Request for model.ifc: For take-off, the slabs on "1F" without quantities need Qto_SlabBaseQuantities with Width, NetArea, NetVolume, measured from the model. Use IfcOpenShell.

First a look at what the model holds.

```python
import ifcopenshell
import ifcopenshell.util.element
import ifcopenshell.util.unit

model = ifcopenshell.open("model.ifc")
print(model.schema)
for unit_type in ("LENGTHUNIT", "AREAUNIT", "VOLUMEUNIT"):
    print(unit_type, ifcopenshell.util.unit.calculate_unit_scale(model, unit_type))
storey = next(s for s in model.by_type("IfcBuildingStorey") if s.Name == "1F")
slabs = [e for e in ifcopenshell.util.element.get_decomposition(storey) if e.is_a("IfcSlab")]
for e in sorted(slabs, key=lambda e: e.id()):
    print(e.id(), e.is_a(), e.Name, list(ifcopenshell.util.element.get_psets(e, qtos_only=True)), sep=" | ")
```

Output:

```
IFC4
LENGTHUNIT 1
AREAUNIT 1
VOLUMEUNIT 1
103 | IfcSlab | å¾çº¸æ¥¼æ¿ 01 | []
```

```python
import ifcopenshell
import ifcopenshell.api.pset
import ifcopenshell.geom
import ifcopenshell.util.element
import ifcopenshell.util.shape
import ifcopenshell.util.unit

model = ifcopenshell.open("model.ifc")
unit_scale = ifcopenshell.util.unit.calculate_unit_scale(model)
area_scale = ifcopenshell.util.unit.calculate_unit_scale(model, "AREAUNIT")
volume_scale = ifcopenshell.util.unit.calculate_unit_scale(model, "VOLUMEUNIT")
settings = ifcopenshell.geom.settings()

storey = next(s for s in model.by_type("IfcBuildingStorey") if s.Name == "1F")
slabs = [e for e in ifcopenshell.util.element.get_decomposition(storey) if e.is_a("IfcSlab")]

for e in sorted(slabs, key=lambda e: e.id()):
    if ifcopenshell.util.element.get_psets(e, qtos_only=True, should_inherit=False):
        continue
    # Geometry comes back in metres, in the element's own axes.
    shape = ifcopenshell.geom.create_shape(settings, e)
    values = {
        "Width": ifcopenshell.util.shape.get_z(shape.geometry) / unit_scale,
        "NetArea": ifcopenshell.util.shape.get_footprint_area(shape.geometry) / area_scale,
        "NetVolume": ifcopenshell.util.shape.get_volume(shape.geometry) / volume_scale,
    }
    qto = ifcopenshell.api.pset.add_qto(model, product=e, name="Qto_SlabBaseQuantities")
    ifcopenshell.api.pset.edit_qto(model, qto=qto, properties=values)
    print(e.id(), {k: round(v, 3) for k, v in values.items()})

model.write("model_v2.ifc")
```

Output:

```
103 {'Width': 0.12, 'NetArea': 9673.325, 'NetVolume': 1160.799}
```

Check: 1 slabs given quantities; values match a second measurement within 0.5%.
